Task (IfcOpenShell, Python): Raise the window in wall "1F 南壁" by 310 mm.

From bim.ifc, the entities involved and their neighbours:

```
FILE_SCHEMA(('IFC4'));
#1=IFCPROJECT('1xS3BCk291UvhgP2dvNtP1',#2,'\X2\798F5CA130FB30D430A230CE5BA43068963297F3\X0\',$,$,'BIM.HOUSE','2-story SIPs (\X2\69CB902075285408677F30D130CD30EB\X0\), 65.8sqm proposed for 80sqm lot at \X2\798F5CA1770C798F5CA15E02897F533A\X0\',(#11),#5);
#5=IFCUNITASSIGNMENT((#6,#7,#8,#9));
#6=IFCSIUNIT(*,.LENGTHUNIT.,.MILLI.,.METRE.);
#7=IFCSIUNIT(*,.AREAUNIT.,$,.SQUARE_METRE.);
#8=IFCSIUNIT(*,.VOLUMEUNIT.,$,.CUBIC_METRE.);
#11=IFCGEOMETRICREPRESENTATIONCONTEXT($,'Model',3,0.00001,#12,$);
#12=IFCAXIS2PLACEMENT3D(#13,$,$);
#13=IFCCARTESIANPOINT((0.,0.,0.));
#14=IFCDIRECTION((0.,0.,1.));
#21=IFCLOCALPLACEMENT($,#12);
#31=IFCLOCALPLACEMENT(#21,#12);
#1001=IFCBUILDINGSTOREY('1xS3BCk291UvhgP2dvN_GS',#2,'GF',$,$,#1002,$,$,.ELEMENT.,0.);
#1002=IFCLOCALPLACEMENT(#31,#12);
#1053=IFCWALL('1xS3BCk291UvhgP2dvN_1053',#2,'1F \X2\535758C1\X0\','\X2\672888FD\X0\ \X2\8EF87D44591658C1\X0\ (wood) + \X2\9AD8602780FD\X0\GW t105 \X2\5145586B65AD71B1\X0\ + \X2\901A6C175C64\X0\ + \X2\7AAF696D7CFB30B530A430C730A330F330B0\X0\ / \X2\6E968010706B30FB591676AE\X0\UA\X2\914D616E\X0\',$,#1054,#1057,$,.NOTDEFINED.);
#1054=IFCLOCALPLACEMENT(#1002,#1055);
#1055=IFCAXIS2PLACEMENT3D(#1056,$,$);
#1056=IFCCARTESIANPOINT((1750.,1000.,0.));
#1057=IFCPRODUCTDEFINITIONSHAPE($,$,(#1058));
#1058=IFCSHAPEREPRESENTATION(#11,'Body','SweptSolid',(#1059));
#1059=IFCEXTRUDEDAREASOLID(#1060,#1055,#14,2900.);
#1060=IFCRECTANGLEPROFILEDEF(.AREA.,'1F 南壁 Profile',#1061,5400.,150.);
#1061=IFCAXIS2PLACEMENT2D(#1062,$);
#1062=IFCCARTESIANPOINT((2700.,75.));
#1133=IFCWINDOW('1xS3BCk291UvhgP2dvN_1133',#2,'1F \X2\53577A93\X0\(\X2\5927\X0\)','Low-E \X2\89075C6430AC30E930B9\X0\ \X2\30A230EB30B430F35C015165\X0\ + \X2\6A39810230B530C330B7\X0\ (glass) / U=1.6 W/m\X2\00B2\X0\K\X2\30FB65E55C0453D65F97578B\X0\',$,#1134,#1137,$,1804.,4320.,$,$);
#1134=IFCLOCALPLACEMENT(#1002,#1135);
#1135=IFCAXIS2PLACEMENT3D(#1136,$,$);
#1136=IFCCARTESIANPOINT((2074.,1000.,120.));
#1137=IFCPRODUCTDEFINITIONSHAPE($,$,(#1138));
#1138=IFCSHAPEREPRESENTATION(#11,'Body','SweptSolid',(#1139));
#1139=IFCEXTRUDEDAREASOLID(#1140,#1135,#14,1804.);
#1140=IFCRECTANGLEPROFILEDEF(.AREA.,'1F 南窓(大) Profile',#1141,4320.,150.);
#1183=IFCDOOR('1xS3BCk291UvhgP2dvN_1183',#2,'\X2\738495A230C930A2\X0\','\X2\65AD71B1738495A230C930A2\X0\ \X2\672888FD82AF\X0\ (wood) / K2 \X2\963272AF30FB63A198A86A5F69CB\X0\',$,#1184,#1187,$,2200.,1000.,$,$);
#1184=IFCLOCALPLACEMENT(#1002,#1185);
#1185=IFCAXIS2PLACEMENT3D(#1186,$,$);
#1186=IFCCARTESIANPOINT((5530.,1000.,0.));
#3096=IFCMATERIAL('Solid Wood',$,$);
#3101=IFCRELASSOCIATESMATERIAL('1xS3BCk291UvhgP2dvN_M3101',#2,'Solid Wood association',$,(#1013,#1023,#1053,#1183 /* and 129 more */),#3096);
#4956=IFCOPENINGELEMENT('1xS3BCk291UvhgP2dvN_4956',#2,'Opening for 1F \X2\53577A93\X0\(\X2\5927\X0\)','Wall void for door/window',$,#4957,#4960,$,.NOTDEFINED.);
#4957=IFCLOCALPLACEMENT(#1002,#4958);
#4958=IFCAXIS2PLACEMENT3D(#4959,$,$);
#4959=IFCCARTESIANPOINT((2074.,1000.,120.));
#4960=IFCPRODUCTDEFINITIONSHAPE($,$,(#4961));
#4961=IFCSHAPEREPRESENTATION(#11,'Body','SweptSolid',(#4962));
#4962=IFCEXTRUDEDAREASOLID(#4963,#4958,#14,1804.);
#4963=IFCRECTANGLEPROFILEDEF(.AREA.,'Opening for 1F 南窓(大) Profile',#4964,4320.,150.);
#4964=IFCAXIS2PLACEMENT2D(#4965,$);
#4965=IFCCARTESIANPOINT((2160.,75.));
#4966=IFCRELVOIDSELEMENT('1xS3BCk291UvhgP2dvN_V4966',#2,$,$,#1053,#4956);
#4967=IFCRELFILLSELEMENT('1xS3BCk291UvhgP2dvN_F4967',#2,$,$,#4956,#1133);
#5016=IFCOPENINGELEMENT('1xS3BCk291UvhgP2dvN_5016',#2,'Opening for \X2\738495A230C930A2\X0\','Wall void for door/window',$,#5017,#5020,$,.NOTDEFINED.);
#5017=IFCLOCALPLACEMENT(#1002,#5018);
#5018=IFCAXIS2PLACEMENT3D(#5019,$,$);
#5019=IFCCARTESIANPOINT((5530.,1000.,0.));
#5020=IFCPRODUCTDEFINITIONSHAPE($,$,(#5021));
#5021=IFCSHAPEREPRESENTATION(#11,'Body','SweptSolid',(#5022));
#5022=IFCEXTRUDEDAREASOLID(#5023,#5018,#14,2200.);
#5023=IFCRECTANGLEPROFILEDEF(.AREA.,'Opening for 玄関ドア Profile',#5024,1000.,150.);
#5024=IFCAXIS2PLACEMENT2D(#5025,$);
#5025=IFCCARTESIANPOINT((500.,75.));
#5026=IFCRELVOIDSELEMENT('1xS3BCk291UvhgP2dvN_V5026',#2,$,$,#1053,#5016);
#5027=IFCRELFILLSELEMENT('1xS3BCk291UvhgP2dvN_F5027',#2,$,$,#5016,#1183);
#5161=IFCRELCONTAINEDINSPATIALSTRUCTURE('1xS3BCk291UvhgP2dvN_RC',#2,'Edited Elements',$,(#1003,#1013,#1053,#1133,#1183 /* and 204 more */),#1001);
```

```python
import numpy as np
import ifcopenshell
import ifcopenshell.api.geometry
import ifcopenshell.util.placement
import ifcopenshell.util.unit

model = ifcopenshell.open("bim.ifc")
unit_scale = ifcopenshell.util.unit.calculate_unit_scale(model)

window = model.by_guid("1xS3BCk291UvhgP2dvN_1133")
opening = window.FillsVoids[0].RelatingOpeningElement
dz = 0.31 / unit_scale

shift = np.array([0.0, 0.0, dz])
# The window is not placed relative to its opening, so move both.
for product in (opening, window):
    matrix = ifcopenshell.util.placement.get_local_placement(product.ObjectPlacement)
    matrix[:3, 3] += shift
    ifcopenshell.api.geometry.edit_object_placement(model, product=product, matrix=matrix, is_si=False)

print(f"moved by {dz * unit_scale:+.3f} m")

model.write("bim_edited.ifc")
```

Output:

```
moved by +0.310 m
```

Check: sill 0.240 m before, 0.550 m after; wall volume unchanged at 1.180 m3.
